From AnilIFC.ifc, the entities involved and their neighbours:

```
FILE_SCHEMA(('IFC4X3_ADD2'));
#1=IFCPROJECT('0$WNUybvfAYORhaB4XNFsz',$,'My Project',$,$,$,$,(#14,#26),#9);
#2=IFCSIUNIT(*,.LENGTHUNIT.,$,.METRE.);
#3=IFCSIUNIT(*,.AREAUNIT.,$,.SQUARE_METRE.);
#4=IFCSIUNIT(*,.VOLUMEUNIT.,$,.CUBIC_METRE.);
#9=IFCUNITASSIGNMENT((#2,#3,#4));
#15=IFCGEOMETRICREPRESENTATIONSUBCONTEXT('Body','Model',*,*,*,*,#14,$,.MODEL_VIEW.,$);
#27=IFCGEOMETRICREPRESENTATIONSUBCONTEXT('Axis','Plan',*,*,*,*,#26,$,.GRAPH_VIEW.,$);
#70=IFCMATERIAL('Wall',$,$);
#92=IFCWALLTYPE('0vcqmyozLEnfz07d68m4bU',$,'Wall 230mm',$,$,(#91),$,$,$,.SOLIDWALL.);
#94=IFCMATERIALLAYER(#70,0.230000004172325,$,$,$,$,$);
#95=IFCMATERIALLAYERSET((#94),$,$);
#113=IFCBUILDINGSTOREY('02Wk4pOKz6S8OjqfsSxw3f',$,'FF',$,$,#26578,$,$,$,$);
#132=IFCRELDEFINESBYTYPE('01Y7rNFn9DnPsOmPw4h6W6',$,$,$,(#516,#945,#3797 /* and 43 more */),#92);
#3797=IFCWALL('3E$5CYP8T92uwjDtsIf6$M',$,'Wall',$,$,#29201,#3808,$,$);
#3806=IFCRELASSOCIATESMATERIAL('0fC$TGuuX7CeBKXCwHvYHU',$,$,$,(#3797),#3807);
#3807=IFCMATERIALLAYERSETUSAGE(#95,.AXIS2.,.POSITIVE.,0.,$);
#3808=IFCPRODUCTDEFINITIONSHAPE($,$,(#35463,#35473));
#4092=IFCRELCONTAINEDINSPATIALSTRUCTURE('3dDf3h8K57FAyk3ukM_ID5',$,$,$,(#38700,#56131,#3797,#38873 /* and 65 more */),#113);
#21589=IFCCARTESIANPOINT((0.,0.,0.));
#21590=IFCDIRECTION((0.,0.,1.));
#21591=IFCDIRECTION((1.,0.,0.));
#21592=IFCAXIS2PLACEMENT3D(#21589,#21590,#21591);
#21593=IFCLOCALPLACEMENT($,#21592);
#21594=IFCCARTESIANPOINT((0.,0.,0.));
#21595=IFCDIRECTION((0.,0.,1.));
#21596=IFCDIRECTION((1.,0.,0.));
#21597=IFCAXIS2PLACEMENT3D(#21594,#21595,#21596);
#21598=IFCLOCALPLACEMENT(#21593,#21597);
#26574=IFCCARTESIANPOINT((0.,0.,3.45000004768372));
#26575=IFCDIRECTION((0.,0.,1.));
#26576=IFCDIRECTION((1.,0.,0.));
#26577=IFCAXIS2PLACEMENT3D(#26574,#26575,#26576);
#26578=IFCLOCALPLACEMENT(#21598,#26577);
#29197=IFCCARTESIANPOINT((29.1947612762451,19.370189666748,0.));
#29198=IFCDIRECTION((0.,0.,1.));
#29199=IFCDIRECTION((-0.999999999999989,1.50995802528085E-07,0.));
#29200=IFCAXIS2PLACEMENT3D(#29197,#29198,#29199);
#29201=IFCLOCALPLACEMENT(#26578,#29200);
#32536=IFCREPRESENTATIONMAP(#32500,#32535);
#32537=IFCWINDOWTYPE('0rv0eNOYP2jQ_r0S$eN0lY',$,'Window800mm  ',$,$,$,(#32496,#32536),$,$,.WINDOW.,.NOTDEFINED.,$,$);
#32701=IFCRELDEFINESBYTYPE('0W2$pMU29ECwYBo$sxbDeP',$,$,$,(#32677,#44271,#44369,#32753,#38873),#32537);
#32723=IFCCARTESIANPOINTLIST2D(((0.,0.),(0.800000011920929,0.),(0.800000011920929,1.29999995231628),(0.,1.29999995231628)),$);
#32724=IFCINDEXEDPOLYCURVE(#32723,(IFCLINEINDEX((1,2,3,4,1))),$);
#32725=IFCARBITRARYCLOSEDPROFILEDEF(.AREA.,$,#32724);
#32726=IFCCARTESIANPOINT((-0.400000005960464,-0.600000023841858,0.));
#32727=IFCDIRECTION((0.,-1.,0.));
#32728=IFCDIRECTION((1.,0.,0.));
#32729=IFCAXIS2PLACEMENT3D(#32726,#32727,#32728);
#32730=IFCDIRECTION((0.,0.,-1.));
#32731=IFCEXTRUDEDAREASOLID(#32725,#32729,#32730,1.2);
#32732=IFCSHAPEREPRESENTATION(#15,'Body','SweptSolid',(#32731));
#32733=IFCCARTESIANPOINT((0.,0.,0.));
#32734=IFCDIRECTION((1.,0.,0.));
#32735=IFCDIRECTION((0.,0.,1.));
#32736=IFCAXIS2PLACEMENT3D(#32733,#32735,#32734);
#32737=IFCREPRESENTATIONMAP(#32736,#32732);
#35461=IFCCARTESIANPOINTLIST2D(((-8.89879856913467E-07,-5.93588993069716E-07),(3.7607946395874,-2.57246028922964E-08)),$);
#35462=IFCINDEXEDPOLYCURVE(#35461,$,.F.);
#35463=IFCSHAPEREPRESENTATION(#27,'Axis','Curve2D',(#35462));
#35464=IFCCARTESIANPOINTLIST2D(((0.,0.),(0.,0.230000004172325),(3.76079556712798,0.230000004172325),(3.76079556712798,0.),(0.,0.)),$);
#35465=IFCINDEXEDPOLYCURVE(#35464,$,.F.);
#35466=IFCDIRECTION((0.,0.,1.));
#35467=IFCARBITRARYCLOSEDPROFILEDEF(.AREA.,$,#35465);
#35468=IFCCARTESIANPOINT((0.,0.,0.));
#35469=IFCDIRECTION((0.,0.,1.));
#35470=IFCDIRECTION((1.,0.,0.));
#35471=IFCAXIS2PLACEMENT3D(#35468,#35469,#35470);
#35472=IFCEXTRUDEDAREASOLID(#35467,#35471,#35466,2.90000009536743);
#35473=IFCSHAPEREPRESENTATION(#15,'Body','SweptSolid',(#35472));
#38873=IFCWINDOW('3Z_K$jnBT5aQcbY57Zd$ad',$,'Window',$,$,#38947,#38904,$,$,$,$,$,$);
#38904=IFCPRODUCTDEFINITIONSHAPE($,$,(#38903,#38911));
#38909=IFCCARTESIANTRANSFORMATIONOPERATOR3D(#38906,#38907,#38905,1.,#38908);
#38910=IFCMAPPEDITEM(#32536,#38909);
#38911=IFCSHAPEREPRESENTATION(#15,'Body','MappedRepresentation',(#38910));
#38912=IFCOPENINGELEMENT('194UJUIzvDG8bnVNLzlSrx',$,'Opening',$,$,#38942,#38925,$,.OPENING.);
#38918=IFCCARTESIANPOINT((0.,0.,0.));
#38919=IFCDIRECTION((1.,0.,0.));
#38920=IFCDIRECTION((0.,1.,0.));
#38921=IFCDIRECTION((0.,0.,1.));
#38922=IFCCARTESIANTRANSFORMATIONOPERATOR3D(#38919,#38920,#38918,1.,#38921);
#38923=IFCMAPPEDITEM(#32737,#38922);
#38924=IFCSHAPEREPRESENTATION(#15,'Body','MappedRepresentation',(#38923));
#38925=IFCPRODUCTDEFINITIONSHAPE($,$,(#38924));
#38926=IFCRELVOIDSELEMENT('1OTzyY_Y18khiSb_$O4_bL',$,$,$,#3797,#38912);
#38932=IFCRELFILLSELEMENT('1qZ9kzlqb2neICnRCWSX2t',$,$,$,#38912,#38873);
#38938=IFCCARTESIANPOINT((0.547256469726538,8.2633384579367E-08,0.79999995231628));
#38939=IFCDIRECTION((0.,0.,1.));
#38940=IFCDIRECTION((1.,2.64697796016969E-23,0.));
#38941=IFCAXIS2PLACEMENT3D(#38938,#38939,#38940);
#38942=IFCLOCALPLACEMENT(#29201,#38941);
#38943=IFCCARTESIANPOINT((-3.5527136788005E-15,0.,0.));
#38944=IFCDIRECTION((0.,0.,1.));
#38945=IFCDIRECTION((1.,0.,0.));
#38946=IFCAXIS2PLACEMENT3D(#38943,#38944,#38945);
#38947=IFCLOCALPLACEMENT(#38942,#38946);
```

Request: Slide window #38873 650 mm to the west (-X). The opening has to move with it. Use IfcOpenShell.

```python
import ifcopenshell
import ifcopenshell.api.geometry
import ifcopenshell.util.placement

model = ifcopenshell.open("AnilIFC.ifc")

window = model.by_guid("3Z_K$jnBT5aQcbY57Zd$ad")
opening = window.FillsVoids[0].RelatingOpeningElement
wall = opening.VoidsElements[0].RelatingBuildingElement

wall_matrix = ifcopenshell.util.placement.get_local_placement(wall.ObjectPlacement)
shift = wall_matrix[:3, 0] * 0.65
before = ifcopenshell.util.placement.get_local_placement(window.ObjectPlacement)[:3, 3].copy()

# The window is placed relative to its opening, so it follows when the opening moves.
matrix = ifcopenshell.util.placement.get_local_placement(opening.ObjectPlacement)
matrix[:3, 3] += shift
ifcopenshell.api.geometry.edit_object_placement(
    model, product=opening, matrix=matrix, is_si=False, should_transform_children=True
)

after = ifcopenshell.util.placement.get_local_placement(window.ObjectPlacement)[:3, 3]
print("window moved by", (after - before).round(3) + 0.0)

model.write("AnilIFC_updated.ifc")
```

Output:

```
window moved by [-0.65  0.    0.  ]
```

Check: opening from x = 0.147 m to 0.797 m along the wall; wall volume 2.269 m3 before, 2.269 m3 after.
